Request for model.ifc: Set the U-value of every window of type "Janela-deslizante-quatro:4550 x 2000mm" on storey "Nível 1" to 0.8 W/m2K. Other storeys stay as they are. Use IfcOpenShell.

First a look at what the model holds.

```python
import ifcopenshell
import ifcopenshell.util.element

model = ifcopenshell.open("model.ifc")
print(model.schema)
storey = next(s for s in model.by_type("IfcBuildingStorey") if s.Name == "Nível 1")
windows = [e for e in ifcopenshell.util.element.get_decomposition(storey) if e.is_a("IfcWindow")]
seen = {}
for e in windows:
    element_type = ifcopenshell.util.element.get_type(e)
    key = (element_type.Name if element_type != e and element_type else None, ifcopenshell.util.element.get_pset(e, "Pset_WindowCommon", "ThermalTransmittance"))
    seen[key] = seen.get(key, 0) + 1
for (name, value), count in sorted(seen.items(), key=str):
    print(count, "x", name, "|", value)
```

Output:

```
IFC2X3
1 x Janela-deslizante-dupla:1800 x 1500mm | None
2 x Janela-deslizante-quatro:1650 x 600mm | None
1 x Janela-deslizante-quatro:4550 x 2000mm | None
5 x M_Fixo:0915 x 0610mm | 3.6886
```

```python
import ifcopenshell
import ifcopenshell.api.pset
import ifcopenshell.util.element

model = ifcopenshell.open("model.ifc")

storey = next(s for s in model.by_type("IfcBuildingStorey") if s.Name == "Nível 1")
windows = [e for e in ifcopenshell.util.element.get_decomposition(storey) if e.is_a("IfcWindow")]

count = 0
for e in windows:
    element_type = ifcopenshell.util.element.get_type(e)
    if element_type in (None, e) or element_type.Name != "Janela-deslizante-quatro:4550 x 2000mm":
        continue
    # add_pset returns the element's existing set when there is one.
    pset = ifcopenshell.api.pset.add_pset(model, product=e, name="Pset_WindowCommon")
    ifcopenshell.api.pset.edit_pset(model, pset=pset, properties={"ThermalTransmittance": 0.8})
    count += 1

print(count, "windows updated")

model.write("model-out.ifc")
```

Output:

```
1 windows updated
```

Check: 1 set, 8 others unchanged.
